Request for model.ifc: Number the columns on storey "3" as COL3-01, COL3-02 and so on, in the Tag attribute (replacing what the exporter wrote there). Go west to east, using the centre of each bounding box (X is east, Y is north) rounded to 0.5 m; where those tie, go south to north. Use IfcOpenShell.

First a look at what the model holds.

```python
import ifcopenshell
import ifcopenshell.util.element
import ifcopenshell.util.placement

model = ifcopenshell.open("model.ifc")
print(model.schema)
storey = next(s for s in model.by_type("IfcBuildingStorey") if s.Name == "3")
columns = [e for e in ifcopenshell.util.element.get_decomposition(storey) if e.is_a("IfcColumn")]
for e in sorted(columns, key=lambda e: e.id()):
    origin = ifcopenshell.util.placement.get_local_placement(e.ObjectPlacement)[:3, 3]
    print(e.id(), e.Tag, e.Name, origin.round(2) + 0.0, sep=" | ")
```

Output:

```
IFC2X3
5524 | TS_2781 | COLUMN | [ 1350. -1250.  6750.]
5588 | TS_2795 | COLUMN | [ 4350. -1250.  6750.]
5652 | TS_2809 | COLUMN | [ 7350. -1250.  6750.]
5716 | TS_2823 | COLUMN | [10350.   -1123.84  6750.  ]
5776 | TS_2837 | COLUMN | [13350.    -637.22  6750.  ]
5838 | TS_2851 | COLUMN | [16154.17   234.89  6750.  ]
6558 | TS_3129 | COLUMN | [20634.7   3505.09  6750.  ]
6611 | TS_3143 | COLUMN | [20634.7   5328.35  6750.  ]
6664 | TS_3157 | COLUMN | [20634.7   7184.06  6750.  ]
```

```python
import ifcopenshell
import ifcopenshell.geom
import ifcopenshell.util.element
import ifcopenshell.util.shape

model = ifcopenshell.open("model.ifc")
settings = ifcopenshell.geom.settings()
settings.set("use-world-coords", True)


def centre(element):
    shape = ifcopenshell.geom.create_shape(settings, element)
    return ifcopenshell.util.shape.get_bbox_centroid(shape.geometry)


storey = next(s for s in model.by_type("IfcBuildingStorey") if s.Name == "3")
columns = [e for e in ifcopenshell.util.element.get_decomposition(storey) if e.is_a("IfcColumn")]

# Insertion points can sit at a corner or the storey origin, so sort by the geometry (in metres).
centres = {e: centre(e) for e in columns}
columns.sort(key=lambda e: (round(centres[e][0] / 0.5), centres[e][1]))

for i, e in enumerate(columns, start=1):
    number = f"COL3-{i:02d}"
    e.Tag = number
    print(e.id(), number)

model.write("model-out.ifc")
```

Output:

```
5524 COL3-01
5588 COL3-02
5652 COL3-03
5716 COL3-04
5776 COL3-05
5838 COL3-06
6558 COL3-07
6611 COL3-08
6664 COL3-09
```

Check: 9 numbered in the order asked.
